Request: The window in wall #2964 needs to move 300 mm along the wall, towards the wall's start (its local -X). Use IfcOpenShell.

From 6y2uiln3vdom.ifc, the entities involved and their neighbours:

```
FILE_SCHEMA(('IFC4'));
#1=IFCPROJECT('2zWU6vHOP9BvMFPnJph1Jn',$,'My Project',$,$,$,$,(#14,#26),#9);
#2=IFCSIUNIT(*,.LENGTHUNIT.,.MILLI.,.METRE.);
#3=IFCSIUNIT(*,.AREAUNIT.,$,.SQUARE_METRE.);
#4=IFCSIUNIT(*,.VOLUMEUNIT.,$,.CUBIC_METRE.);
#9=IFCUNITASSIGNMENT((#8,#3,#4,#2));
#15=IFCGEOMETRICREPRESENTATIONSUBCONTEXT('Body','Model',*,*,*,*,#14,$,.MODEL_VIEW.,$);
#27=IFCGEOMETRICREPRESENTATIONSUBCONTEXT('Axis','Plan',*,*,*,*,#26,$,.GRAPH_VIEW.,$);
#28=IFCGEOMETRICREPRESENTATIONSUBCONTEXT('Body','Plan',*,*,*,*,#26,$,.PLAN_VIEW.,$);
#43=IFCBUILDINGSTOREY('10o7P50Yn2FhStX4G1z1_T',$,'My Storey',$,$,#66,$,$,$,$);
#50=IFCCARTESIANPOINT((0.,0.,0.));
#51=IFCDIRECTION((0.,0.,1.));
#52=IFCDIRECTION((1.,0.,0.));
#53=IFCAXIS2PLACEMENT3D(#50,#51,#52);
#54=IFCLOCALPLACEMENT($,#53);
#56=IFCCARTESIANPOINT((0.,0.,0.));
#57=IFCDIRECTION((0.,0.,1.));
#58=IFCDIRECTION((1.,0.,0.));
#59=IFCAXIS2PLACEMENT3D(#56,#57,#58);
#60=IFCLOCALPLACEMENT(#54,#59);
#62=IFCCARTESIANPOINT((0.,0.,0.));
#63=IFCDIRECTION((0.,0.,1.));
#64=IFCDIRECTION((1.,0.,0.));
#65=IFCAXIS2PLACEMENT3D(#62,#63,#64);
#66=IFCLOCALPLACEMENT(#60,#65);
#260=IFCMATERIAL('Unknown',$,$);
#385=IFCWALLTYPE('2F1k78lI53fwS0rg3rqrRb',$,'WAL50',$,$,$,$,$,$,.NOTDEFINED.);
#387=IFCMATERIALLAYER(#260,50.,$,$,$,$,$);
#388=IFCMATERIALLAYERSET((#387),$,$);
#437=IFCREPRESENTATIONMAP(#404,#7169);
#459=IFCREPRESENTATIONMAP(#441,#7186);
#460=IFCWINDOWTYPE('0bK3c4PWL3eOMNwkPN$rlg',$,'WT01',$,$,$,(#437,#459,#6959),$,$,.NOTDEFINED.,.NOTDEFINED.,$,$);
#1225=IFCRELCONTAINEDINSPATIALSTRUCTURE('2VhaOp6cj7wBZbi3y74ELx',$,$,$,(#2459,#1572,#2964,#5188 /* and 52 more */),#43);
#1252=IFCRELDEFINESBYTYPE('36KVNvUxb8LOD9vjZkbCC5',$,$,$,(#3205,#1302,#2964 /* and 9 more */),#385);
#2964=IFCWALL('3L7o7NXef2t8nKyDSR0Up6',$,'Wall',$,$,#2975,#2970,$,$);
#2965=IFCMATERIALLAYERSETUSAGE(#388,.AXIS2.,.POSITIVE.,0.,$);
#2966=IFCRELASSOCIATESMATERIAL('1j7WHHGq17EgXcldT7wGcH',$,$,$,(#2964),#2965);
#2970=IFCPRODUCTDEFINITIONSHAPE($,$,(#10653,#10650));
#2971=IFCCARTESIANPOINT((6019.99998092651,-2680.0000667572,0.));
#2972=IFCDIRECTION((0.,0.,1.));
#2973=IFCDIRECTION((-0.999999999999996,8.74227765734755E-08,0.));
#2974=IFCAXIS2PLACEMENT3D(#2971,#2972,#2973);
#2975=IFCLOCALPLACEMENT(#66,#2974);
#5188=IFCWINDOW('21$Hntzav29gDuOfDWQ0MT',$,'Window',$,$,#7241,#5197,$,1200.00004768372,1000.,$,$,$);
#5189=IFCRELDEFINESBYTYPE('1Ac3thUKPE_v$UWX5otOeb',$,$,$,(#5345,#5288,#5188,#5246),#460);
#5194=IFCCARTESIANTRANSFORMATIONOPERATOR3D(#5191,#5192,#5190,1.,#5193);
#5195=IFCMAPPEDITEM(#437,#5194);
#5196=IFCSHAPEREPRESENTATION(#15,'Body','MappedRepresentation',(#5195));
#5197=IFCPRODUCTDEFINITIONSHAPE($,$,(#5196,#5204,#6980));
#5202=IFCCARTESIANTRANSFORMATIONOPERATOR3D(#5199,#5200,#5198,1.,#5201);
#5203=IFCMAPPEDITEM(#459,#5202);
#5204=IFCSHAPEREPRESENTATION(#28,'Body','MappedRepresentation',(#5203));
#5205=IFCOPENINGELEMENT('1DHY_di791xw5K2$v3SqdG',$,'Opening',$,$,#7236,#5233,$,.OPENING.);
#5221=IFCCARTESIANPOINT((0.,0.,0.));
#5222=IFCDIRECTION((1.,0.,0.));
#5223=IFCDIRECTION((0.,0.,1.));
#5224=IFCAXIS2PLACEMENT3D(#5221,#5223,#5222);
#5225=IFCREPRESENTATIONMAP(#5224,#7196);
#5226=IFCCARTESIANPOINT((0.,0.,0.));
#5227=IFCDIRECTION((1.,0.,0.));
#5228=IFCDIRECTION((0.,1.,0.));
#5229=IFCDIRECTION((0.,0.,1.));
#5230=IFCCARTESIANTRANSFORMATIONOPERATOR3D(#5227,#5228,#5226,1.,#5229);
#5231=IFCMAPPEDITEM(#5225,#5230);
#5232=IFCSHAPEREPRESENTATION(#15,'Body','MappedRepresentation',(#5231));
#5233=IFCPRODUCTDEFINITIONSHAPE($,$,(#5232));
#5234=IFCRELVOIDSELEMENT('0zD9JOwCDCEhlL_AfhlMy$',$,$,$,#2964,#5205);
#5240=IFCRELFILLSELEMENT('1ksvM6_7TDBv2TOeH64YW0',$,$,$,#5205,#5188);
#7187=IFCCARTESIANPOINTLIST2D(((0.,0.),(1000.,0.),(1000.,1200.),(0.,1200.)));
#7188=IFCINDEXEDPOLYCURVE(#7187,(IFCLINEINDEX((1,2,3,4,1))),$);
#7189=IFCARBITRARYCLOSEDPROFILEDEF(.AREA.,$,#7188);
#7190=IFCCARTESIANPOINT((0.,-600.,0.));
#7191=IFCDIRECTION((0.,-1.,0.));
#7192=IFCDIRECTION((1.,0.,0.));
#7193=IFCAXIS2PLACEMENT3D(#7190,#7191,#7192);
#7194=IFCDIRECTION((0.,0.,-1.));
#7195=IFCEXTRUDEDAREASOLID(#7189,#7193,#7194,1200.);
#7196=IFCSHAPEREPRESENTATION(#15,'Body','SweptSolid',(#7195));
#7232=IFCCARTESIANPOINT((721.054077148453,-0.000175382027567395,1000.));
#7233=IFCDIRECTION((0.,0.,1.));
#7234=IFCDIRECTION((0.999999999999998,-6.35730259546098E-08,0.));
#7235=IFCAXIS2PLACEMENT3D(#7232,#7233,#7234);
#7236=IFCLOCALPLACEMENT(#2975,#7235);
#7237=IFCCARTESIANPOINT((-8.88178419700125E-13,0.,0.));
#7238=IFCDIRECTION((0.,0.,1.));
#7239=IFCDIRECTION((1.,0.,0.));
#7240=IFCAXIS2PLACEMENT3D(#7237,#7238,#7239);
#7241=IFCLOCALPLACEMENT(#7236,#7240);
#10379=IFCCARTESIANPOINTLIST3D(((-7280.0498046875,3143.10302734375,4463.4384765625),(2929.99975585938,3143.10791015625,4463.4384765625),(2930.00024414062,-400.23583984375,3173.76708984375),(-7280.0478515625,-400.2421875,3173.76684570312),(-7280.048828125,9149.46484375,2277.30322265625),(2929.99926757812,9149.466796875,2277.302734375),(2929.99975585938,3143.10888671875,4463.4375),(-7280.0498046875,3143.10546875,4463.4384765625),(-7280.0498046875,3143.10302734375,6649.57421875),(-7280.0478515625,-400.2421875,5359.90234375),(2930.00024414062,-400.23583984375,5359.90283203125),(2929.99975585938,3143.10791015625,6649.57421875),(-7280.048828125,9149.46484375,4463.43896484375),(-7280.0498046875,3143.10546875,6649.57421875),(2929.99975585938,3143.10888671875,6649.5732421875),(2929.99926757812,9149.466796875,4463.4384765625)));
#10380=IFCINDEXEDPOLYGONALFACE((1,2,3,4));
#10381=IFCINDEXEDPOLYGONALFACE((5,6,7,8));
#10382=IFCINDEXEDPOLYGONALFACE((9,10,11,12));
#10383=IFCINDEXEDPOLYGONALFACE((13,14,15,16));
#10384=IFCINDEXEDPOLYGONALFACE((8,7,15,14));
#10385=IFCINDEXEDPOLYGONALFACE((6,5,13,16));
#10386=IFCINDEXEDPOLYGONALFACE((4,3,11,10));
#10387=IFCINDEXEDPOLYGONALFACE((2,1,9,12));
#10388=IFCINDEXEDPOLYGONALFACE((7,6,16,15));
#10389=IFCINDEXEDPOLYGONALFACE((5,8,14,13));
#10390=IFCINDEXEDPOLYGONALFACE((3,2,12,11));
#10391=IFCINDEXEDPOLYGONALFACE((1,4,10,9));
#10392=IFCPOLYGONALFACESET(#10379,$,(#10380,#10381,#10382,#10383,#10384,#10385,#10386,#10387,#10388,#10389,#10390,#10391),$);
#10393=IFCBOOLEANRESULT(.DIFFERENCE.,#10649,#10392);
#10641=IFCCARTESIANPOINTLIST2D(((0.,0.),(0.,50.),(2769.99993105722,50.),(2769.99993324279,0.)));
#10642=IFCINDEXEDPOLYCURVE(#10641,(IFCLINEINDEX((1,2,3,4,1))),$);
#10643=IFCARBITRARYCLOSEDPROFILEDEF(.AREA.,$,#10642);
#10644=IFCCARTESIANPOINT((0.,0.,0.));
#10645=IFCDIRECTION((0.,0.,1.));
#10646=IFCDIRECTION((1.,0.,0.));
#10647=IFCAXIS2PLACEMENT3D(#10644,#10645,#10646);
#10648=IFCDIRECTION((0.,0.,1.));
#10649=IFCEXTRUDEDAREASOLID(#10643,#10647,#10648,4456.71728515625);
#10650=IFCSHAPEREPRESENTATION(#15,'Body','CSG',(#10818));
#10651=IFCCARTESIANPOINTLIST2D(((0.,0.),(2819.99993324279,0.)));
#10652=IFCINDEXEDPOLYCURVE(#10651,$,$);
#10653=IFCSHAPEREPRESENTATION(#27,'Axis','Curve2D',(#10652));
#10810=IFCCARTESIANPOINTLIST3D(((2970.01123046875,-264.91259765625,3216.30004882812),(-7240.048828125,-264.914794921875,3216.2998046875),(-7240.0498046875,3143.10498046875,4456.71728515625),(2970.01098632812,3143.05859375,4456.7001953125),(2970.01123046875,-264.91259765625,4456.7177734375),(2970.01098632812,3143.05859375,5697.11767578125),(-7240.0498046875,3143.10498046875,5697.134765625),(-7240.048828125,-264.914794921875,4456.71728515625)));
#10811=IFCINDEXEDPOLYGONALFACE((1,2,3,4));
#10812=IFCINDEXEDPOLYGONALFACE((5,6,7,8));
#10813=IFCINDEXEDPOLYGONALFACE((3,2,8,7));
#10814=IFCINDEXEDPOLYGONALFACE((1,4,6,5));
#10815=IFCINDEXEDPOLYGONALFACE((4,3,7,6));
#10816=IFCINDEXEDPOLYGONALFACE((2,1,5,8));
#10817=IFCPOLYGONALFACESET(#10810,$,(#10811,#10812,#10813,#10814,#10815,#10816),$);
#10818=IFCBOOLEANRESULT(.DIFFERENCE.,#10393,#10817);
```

```python
import ifcopenshell
import ifcopenshell.api.geometry
import ifcopenshell.util.placement
import ifcopenshell.util.unit

model = ifcopenshell.open("6y2uiln3vdom.ifc")
unit_scale = ifcopenshell.util.unit.calculate_unit_scale(model)

window = model.by_guid("21$Hntzav29gDuOfDWQ0MT")
opening = window.FillsVoids[0].RelatingOpeningElement
wall = opening.VoidsElements[0].RelatingBuildingElement

wall_matrix = ifcopenshell.util.placement.get_local_placement(wall.ObjectPlacement)
shift = wall_matrix[:3, 0] * -0.3 / unit_scale
before = ifcopenshell.util.placement.get_local_placement(window.ObjectPlacement)[:3, 3].copy()

# The window is placed relative to its opening, so it follows when the opening moves.
matrix = ifcopenshell.util.placement.get_local_placement(opening.ObjectPlacement)
matrix[:3, 3] += shift
ifcopenshell.api.geometry.edit_object_placement(
    model, product=opening, matrix=matrix, is_si=False, should_transform_children=True
)

after = ifcopenshell.util.placement.get_local_placement(window.ObjectPlacement)[:3, 3]
print("window moved by", (after - before).round(3) + 0.0)

model.write("6y2uiln3vdom-out.ifc")
```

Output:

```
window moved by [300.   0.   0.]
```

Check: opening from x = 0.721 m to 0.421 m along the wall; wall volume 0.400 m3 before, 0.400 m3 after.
